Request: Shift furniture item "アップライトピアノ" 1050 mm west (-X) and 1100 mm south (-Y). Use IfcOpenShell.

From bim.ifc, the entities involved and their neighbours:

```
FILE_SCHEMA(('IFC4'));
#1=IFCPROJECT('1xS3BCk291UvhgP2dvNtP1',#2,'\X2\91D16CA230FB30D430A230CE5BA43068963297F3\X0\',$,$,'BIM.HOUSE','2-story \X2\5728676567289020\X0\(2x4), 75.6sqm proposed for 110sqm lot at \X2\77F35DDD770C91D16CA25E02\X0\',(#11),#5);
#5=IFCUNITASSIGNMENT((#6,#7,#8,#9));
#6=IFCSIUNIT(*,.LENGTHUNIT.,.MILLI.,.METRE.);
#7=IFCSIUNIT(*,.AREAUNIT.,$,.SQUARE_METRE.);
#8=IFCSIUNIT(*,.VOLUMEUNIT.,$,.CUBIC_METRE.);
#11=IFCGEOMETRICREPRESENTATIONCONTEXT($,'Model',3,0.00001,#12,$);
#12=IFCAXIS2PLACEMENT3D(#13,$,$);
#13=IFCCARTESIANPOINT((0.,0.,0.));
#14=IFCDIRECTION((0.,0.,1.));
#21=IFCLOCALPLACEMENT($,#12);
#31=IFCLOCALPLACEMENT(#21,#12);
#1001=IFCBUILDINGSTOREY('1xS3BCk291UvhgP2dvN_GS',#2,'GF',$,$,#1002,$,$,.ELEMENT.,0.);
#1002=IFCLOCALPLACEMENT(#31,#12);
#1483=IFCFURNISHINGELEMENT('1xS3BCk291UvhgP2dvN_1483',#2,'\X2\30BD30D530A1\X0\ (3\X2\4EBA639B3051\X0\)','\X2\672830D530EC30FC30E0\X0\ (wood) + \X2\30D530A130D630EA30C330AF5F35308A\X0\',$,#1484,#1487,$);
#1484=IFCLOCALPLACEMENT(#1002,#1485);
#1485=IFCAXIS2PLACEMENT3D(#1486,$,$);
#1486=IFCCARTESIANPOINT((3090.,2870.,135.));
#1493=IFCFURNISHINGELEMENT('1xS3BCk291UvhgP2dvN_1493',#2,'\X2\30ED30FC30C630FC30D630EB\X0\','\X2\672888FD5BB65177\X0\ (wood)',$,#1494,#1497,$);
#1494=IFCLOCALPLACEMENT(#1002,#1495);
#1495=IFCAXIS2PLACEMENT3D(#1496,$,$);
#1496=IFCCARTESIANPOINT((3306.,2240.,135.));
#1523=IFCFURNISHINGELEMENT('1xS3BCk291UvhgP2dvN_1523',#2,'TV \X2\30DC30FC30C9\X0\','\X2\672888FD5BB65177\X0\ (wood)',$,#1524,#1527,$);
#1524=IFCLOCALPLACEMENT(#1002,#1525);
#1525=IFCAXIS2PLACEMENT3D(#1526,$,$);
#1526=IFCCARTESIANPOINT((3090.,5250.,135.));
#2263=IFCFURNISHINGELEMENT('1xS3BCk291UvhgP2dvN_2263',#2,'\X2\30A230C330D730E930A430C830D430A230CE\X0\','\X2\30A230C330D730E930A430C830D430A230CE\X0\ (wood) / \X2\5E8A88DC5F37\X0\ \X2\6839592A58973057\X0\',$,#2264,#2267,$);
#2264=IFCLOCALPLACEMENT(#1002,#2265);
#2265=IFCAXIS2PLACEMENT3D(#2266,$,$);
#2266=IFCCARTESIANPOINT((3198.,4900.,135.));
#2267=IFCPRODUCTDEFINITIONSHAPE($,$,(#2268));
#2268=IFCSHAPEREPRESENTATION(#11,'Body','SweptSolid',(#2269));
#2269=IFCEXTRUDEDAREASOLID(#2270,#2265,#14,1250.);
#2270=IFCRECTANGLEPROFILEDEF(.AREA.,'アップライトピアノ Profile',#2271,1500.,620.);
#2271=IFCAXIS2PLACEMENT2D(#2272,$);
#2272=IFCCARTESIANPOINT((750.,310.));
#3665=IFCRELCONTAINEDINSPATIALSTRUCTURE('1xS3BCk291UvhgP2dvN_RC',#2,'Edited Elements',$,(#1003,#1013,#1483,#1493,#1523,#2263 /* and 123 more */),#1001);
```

```python
import ifcopenshell
import ifcopenshell.api.geometry
import ifcopenshell.util.placement

model = ifcopenshell.open("bim.ifc")

item = model.by_guid("1xS3BCk291UvhgP2dvN_2263")
matrix = ifcopenshell.util.placement.get_local_placement(item.ObjectPlacement)
matrix[0, 3] -= 1050.0
matrix[1, 3] -= 1100.0
ifcopenshell.api.geometry.edit_object_placement(model, product=item, matrix=matrix, is_si=False)

print(ifcopenshell.util.placement.get_local_placement(item.ObjectPlacement).round(3) + 0.0)

model.write("bim_v2.ifc")
```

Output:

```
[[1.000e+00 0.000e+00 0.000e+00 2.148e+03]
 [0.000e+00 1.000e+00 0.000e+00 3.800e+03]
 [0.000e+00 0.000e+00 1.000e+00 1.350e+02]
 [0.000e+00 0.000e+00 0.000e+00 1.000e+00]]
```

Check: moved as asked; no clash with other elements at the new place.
